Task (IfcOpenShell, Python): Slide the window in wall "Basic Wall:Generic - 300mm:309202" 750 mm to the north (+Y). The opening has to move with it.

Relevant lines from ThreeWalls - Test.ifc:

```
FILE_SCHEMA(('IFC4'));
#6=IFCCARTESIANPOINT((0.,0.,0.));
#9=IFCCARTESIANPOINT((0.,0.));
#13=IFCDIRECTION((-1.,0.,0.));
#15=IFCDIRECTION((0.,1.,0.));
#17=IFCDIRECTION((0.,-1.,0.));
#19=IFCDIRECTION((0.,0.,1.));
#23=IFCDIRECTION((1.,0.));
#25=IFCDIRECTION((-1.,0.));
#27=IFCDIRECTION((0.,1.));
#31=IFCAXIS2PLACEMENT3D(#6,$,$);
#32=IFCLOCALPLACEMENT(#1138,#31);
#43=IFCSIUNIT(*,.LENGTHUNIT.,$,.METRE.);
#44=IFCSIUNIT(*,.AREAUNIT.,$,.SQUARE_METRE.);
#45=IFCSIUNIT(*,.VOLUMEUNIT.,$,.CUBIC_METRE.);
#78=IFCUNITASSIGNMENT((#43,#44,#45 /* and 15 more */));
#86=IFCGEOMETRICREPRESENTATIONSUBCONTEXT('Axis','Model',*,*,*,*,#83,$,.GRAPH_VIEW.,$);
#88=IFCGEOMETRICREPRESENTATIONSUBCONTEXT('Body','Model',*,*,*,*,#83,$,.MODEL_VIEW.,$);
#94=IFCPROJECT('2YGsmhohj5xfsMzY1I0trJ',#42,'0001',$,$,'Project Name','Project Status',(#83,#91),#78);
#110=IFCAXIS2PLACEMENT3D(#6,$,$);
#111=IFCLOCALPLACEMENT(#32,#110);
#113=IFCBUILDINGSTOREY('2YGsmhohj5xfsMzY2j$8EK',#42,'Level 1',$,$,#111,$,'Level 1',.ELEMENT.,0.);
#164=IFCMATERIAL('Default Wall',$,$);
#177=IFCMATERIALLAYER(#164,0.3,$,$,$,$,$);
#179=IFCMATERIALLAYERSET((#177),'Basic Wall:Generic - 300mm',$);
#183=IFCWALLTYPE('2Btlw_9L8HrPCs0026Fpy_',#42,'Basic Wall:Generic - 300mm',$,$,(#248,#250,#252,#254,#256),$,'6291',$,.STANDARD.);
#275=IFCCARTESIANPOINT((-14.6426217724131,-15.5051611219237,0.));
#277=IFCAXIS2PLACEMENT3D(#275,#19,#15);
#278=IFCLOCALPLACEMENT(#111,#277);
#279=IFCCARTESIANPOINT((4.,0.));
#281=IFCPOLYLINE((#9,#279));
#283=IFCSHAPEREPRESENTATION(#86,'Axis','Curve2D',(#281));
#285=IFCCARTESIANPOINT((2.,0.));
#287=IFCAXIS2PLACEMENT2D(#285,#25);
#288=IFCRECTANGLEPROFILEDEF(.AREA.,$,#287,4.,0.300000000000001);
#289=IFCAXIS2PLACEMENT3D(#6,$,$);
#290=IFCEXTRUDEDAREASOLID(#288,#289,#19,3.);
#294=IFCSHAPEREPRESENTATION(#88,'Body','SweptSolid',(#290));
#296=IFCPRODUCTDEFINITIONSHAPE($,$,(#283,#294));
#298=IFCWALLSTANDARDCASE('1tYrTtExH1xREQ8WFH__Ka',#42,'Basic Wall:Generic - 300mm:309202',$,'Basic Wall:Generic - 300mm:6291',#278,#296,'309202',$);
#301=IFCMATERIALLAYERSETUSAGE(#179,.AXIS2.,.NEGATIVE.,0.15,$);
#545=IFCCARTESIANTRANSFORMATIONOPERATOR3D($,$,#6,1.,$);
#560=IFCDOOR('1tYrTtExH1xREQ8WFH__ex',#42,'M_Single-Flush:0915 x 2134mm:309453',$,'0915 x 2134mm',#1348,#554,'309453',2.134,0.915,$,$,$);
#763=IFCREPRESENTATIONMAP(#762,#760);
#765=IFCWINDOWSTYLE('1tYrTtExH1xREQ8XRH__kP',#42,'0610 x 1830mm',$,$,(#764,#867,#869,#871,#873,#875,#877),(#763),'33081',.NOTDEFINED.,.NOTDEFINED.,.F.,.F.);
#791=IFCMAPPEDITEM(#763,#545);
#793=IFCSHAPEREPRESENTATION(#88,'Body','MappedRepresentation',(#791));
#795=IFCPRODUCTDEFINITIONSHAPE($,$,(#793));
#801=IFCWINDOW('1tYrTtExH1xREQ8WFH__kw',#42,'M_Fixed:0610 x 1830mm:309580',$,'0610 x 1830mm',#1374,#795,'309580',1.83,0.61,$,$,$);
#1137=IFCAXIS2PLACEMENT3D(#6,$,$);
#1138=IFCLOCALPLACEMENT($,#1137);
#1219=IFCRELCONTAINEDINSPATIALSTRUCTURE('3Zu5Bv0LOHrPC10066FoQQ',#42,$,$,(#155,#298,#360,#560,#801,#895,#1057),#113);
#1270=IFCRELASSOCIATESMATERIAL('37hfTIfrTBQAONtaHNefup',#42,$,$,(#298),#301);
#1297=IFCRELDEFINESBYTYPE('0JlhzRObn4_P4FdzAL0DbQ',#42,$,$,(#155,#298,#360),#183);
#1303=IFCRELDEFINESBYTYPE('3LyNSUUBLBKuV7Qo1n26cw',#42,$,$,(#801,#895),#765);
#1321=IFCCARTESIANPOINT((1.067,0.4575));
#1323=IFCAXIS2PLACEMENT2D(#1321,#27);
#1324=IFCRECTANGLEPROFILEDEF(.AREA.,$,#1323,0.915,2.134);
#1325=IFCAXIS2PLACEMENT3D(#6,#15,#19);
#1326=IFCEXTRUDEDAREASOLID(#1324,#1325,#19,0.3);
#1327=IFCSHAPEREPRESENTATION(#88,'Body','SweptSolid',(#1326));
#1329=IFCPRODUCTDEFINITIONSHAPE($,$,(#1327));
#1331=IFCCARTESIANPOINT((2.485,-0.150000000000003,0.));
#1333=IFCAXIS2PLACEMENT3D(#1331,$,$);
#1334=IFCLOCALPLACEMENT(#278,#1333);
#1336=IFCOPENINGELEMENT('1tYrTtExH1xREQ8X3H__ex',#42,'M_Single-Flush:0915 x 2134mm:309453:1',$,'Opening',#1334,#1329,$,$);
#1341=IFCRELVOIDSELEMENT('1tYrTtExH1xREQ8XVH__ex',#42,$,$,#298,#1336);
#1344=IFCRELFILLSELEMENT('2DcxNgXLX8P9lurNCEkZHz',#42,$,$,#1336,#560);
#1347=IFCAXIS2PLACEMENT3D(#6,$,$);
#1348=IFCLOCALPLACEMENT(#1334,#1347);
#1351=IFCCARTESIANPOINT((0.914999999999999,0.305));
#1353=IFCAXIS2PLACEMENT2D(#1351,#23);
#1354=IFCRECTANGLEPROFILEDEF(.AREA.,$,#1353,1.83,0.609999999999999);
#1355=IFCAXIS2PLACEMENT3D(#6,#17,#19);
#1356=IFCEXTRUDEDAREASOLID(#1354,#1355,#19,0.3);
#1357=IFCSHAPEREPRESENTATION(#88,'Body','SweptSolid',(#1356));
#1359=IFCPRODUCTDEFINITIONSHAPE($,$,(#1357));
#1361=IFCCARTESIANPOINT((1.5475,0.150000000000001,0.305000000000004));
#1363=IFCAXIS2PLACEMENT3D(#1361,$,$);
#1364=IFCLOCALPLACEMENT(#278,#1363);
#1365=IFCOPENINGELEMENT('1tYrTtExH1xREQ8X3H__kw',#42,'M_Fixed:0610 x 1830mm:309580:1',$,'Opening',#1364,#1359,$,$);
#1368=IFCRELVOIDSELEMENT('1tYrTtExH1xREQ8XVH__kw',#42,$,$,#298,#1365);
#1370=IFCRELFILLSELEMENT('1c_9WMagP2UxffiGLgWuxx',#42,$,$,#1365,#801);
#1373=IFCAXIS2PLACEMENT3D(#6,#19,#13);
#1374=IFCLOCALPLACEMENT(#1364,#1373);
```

```python
import ifcopenshell
import ifcopenshell.api.geometry
import ifcopenshell.util.placement

model = ifcopenshell.open("ThreeWalls - Test.ifc")

window = model.by_guid("1tYrTtExH1xREQ8WFH__kw")
opening = window.FillsVoids[0].RelatingOpeningElement
wall = opening.VoidsElements[0].RelatingBuildingElement

wall_matrix = ifcopenshell.util.placement.get_local_placement(wall.ObjectPlacement)
shift = wall_matrix[:3, 0] * 0.75
before = ifcopenshell.util.placement.get_local_placement(window.ObjectPlacement)[:3, 3].copy()

# The window is placed relative to its opening, so it follows when the opening moves.
matrix = ifcopenshell.util.placement.get_local_placement(opening.ObjectPlacement)
matrix[:3, 3] += shift
ifcopenshell.api.geometry.edit_object_placement(
    model, product=opening, matrix=matrix, is_si=False, should_transform_children=True
)

after = ifcopenshell.util.placement.get_local_placement(window.ObjectPlacement)[:3, 3]
print("window moved by", (after - before).round(3) + 0.0)

model.write("ThreeWalls - Test_edited.ifc")
```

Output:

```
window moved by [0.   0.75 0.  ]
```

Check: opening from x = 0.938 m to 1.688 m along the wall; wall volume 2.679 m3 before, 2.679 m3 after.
